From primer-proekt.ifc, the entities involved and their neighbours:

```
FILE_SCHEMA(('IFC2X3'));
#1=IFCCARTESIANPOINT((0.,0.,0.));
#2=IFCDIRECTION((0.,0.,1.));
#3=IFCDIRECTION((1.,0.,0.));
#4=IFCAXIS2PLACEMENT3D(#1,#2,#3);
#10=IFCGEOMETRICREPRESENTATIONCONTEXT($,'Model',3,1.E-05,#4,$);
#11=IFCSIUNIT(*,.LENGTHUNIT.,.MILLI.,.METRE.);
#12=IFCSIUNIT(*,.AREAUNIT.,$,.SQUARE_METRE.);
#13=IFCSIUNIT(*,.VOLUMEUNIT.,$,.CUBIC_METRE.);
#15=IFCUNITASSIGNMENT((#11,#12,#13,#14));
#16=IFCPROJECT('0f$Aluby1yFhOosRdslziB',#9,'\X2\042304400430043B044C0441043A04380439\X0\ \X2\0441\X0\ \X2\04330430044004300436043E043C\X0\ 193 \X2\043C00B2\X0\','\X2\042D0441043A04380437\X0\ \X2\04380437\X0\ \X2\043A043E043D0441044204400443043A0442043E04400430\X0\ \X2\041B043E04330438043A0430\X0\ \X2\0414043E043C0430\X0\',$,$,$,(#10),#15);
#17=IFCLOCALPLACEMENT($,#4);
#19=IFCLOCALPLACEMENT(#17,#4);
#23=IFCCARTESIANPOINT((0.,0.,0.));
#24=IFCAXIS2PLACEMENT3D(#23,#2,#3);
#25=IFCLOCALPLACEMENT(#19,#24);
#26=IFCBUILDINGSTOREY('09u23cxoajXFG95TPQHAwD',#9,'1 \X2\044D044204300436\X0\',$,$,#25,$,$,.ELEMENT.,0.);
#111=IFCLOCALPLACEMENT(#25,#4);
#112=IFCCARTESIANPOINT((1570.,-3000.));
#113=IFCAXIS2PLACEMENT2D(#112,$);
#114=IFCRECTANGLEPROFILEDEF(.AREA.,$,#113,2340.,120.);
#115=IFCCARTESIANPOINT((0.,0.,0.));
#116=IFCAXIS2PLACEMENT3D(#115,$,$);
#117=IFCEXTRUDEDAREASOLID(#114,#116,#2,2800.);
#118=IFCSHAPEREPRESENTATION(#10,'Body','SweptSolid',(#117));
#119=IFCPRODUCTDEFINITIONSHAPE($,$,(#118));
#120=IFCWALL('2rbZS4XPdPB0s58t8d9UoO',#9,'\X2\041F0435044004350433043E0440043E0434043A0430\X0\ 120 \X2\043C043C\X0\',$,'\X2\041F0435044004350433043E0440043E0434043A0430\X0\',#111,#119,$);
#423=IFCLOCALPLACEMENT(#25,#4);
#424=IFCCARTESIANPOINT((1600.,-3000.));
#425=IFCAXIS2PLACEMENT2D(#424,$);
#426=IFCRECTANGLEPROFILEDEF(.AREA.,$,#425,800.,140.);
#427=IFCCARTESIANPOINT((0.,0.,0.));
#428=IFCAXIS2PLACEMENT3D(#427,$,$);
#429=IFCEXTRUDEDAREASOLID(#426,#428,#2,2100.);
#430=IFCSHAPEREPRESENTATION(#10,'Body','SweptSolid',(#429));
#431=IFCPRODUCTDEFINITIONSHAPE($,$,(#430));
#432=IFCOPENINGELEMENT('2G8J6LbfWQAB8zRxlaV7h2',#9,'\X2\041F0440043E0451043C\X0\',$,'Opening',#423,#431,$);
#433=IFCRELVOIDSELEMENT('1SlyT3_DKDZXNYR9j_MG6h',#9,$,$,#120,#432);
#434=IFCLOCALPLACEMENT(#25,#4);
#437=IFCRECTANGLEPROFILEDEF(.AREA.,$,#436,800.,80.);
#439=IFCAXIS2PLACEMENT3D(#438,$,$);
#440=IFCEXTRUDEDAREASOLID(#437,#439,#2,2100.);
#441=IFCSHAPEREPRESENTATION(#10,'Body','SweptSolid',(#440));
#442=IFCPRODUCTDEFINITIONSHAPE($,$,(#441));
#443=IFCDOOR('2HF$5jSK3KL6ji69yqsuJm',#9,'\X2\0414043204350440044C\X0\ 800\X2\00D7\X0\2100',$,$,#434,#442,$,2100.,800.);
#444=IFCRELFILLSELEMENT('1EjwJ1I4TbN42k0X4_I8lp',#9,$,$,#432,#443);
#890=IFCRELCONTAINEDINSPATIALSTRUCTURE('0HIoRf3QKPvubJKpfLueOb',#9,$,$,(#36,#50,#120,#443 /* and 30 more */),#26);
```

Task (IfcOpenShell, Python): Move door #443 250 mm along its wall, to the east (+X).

```python
import ifcopenshell
import ifcopenshell.api.geometry
import ifcopenshell.util.placement
import ifcopenshell.util.unit

model = ifcopenshell.open("primer-proekt.ifc")
unit_scale = ifcopenshell.util.unit.calculate_unit_scale(model)

door = model.by_id(443)
opening = door.FillsVoids[0].RelatingOpeningElement
wall = opening.VoidsElements[0].RelatingBuildingElement

wall_matrix = ifcopenshell.util.placement.get_local_placement(wall.ObjectPlacement)
shift = wall_matrix[:3, 0] * 0.25 / unit_scale
before = ifcopenshell.util.placement.get_local_placement(door.ObjectPlacement)[:3, 3].copy()

# The door is not placed relative to its opening, so move both.
for product in (opening, door):
    matrix = ifcopenshell.util.placement.get_local_placement(product.ObjectPlacement)
    matrix[:3, 3] += shift
    ifcopenshell.api.geometry.edit_object_placement(model, product=product, matrix=matrix, is_si=False)

after = ifcopenshell.util.placement.get_local_placement(door.ObjectPlacement)[:3, 3]
print("door moved by", (after - before).round(3) + 0.0)

model.write("primer-proekt_rev.ifc")
```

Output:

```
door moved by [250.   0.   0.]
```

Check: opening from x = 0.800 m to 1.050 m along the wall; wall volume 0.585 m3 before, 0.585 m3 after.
